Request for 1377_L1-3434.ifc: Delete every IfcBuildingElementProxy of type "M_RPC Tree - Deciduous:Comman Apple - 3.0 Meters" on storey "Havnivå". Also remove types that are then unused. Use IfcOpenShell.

First a look at what the model holds.

```python
import ifcopenshell
import ifcopenshell.util.element

model = ifcopenshell.open("1377_L1-3434.ifc")
print(model.schema)
storey = next(s for s in model.by_type("IfcBuildingStorey") if s.Name == "Havnivå")
proxies = [e for e in ifcopenshell.util.element.get_decomposition(storey) if e.is_a("IfcBuildingElementProxy")]
seen = {}
for e in proxies:
    element_type = ifcopenshell.util.element.get_type(e)
    name = element_type.Name if element_type not in (None, e) else None
    seen[name] = seen.get(name, 0) + 1
for name, count in sorted(seen.items(), key=str):
    print(count, "x", name)
```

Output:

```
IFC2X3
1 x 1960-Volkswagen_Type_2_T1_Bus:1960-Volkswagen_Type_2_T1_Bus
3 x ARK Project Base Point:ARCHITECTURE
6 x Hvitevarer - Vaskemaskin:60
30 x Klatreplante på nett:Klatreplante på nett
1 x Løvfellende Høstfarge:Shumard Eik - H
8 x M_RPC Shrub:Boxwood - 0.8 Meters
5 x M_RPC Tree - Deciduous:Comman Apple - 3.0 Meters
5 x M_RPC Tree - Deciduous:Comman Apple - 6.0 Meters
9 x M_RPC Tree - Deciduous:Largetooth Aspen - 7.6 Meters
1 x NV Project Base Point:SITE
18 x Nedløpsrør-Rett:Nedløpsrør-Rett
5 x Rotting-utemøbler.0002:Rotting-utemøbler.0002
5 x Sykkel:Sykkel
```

```python
import ifcopenshell
import ifcopenshell.api.root
import ifcopenshell.util.element

model = ifcopenshell.open("1377_L1-3434.ifc")

storey = next(s for s in model.by_type("IfcBuildingStorey") if s.Name == "Havnivå")
proxies = [e for e in ifcopenshell.util.element.get_decomposition(storey) if e.is_a("IfcBuildingElementProxy")]
targets = [e for e in proxies if (t := ifcopenshell.util.element.get_type(e)) not in (None, e) and t.Name == "M_RPC Tree - Deciduous:Comman Apple - 3.0 Meters"]
types = {ifcopenshell.util.element.get_type(e) for e in targets} - {None, *targets}

for e in targets:
    ifcopenshell.api.root.remove_product(model, product=e)
print(len(targets), "removed")

unused = [t for t in types if not ifcopenshell.util.element.get_types(t)]
for t in unused:
    ifcopenshell.api.root.remove_product(model, product=t)
print(len(unused), "unused types removed")

model.write("1377_L1-3434_updated.ifc")
```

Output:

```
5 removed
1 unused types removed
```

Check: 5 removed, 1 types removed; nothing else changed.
